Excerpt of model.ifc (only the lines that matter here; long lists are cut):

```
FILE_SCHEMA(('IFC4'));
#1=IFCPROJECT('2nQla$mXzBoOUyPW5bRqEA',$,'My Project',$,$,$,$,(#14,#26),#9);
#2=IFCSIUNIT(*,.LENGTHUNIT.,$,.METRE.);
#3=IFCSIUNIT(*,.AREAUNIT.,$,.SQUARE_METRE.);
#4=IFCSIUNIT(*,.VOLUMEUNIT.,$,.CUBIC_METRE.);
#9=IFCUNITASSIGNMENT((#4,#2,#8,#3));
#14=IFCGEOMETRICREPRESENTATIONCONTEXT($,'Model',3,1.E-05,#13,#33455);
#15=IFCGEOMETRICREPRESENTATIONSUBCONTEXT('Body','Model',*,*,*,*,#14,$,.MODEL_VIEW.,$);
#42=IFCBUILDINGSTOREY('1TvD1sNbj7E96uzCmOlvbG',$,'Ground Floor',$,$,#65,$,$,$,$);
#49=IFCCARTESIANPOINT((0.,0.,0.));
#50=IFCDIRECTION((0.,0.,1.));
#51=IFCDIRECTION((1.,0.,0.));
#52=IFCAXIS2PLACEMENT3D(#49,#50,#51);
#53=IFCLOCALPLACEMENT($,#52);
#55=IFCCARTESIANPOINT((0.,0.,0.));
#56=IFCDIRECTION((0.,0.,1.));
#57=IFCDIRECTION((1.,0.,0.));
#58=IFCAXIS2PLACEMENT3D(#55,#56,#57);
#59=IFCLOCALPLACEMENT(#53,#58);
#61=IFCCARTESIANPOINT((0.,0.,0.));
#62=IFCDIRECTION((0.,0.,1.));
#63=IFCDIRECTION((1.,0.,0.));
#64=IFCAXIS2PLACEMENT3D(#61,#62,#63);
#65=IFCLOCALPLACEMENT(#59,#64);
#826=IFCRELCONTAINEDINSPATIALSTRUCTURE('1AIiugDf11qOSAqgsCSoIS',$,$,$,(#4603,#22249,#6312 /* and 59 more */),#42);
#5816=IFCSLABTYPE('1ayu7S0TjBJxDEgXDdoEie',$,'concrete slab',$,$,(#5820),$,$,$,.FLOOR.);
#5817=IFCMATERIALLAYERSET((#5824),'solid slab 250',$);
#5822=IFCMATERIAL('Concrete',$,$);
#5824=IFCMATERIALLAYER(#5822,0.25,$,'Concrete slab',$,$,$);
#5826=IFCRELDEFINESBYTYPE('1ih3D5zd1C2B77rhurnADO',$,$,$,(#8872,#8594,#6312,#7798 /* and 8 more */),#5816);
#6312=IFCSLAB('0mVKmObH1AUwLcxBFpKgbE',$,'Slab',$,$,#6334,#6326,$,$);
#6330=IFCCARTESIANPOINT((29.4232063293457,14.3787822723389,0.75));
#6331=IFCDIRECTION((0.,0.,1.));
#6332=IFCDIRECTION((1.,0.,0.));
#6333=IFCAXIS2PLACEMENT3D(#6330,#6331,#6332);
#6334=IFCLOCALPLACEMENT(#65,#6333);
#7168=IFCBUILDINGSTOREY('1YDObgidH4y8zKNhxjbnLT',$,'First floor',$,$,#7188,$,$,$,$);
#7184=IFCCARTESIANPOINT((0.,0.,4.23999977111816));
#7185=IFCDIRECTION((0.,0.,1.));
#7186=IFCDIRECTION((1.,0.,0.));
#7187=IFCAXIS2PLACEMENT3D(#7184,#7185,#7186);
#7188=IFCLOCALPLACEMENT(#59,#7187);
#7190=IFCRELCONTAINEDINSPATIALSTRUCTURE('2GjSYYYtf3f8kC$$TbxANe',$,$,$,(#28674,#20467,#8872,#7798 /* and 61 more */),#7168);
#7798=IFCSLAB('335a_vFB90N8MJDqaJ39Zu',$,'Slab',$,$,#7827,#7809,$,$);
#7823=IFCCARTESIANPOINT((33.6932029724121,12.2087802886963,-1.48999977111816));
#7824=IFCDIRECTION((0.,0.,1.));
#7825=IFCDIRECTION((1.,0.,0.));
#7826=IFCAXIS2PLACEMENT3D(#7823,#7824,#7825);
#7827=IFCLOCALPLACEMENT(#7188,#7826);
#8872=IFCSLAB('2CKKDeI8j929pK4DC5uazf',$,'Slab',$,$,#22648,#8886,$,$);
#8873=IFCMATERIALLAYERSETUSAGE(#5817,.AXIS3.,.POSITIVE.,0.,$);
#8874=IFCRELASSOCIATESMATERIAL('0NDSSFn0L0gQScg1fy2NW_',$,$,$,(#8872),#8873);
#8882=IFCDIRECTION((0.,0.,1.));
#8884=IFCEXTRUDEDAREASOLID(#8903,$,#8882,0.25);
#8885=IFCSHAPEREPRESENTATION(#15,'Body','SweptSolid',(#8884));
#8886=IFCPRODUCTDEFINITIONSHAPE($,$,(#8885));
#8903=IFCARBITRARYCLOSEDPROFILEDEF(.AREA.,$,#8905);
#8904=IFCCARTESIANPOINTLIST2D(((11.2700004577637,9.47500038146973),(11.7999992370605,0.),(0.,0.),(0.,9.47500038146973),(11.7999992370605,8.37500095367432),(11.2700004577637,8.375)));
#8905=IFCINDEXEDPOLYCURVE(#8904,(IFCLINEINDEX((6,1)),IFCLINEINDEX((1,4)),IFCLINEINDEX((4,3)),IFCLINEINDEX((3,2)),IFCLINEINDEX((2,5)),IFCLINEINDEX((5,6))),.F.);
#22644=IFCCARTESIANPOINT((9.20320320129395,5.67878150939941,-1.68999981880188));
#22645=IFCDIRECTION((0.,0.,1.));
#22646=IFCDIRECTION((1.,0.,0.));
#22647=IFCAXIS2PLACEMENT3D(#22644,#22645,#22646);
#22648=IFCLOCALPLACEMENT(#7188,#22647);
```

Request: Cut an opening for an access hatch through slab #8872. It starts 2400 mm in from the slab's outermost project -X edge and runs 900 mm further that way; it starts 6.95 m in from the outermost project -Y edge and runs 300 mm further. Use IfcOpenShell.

```python
import numpy as np
import ifcopenshell
import ifcopenshell.api.feature
import ifcopenshell.api.geometry
import ifcopenshell.api.root
import ifcopenshell.geom
import ifcopenshell.util.placement
import ifcopenshell.util.representation
import ifcopenshell.util.shape
import ifcopenshell.util.unit

model = ifcopenshell.open("model.ifc")
unit_scale = ifcopenshell.util.unit.calculate_unit_scale(model)
settings = ifcopenshell.geom.settings()


def volume(element):
    """Net volume in cubic metres, openings subtracted."""
    shape = ifcopenshell.geom.create_shape(settings, element)
    return ifcopenshell.util.shape.get_volume(shape.geometry)


slab = model.by_id(8872)
before = volume(slab)

# Extent in the slab's own axes, in metres. The edges named are its -X and -Y sides.
slab_shape = ifcopenshell.geom.create_shape(settings, slab)
vertices = ifcopenshell.util.shape.get_vertices(slab_shape.geometry)
x_min, y_min, bottom = vertices.min(axis=0)
top = vertices[:, 2].max()

opening = ifcopenshell.api.root.create_entity(model, ifc_class="IfcOpeningElement", name="Access hatch opening", predefined_type="OPENING")
context = ifcopenshell.util.representation.get_context(model, "Model", "Body", "MODEL_VIEW")
width, depth = 0.9, 0.3
outline = [(0.0, 0.0), (width, 0.0), (width, depth), (0.0, depth), (0.0, 0.0)]
# Overshoot both faces by 50 mm so the cut is clean.
shape = ifcopenshell.api.geometry.add_slab_representation(
    model, context=context, depth=top - bottom + 0.1, polyline=outline
)
ifcopenshell.api.geometry.assign_representation(model, product=opening, representation=shape)

matrix = ifcopenshell.util.placement.get_local_placement(slab.ObjectPlacement)
matrix[:, 3] = matrix @ np.append(np.array([x_min + 2.4, y_min + 6.95, bottom - 0.05]) / unit_scale, 1.0)
ifcopenshell.api.geometry.edit_object_placement(model, product=opening, matrix=matrix, is_si=False)
ifcopenshell.api.feature.add_feature(model, feature=opening, element=slab)

after = volume(slab)

print(f"slab volume {before:.3f} -> {after:.3f} m3")

model.write("model_edited.ifc")
```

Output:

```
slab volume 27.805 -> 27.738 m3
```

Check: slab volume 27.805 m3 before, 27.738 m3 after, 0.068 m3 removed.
